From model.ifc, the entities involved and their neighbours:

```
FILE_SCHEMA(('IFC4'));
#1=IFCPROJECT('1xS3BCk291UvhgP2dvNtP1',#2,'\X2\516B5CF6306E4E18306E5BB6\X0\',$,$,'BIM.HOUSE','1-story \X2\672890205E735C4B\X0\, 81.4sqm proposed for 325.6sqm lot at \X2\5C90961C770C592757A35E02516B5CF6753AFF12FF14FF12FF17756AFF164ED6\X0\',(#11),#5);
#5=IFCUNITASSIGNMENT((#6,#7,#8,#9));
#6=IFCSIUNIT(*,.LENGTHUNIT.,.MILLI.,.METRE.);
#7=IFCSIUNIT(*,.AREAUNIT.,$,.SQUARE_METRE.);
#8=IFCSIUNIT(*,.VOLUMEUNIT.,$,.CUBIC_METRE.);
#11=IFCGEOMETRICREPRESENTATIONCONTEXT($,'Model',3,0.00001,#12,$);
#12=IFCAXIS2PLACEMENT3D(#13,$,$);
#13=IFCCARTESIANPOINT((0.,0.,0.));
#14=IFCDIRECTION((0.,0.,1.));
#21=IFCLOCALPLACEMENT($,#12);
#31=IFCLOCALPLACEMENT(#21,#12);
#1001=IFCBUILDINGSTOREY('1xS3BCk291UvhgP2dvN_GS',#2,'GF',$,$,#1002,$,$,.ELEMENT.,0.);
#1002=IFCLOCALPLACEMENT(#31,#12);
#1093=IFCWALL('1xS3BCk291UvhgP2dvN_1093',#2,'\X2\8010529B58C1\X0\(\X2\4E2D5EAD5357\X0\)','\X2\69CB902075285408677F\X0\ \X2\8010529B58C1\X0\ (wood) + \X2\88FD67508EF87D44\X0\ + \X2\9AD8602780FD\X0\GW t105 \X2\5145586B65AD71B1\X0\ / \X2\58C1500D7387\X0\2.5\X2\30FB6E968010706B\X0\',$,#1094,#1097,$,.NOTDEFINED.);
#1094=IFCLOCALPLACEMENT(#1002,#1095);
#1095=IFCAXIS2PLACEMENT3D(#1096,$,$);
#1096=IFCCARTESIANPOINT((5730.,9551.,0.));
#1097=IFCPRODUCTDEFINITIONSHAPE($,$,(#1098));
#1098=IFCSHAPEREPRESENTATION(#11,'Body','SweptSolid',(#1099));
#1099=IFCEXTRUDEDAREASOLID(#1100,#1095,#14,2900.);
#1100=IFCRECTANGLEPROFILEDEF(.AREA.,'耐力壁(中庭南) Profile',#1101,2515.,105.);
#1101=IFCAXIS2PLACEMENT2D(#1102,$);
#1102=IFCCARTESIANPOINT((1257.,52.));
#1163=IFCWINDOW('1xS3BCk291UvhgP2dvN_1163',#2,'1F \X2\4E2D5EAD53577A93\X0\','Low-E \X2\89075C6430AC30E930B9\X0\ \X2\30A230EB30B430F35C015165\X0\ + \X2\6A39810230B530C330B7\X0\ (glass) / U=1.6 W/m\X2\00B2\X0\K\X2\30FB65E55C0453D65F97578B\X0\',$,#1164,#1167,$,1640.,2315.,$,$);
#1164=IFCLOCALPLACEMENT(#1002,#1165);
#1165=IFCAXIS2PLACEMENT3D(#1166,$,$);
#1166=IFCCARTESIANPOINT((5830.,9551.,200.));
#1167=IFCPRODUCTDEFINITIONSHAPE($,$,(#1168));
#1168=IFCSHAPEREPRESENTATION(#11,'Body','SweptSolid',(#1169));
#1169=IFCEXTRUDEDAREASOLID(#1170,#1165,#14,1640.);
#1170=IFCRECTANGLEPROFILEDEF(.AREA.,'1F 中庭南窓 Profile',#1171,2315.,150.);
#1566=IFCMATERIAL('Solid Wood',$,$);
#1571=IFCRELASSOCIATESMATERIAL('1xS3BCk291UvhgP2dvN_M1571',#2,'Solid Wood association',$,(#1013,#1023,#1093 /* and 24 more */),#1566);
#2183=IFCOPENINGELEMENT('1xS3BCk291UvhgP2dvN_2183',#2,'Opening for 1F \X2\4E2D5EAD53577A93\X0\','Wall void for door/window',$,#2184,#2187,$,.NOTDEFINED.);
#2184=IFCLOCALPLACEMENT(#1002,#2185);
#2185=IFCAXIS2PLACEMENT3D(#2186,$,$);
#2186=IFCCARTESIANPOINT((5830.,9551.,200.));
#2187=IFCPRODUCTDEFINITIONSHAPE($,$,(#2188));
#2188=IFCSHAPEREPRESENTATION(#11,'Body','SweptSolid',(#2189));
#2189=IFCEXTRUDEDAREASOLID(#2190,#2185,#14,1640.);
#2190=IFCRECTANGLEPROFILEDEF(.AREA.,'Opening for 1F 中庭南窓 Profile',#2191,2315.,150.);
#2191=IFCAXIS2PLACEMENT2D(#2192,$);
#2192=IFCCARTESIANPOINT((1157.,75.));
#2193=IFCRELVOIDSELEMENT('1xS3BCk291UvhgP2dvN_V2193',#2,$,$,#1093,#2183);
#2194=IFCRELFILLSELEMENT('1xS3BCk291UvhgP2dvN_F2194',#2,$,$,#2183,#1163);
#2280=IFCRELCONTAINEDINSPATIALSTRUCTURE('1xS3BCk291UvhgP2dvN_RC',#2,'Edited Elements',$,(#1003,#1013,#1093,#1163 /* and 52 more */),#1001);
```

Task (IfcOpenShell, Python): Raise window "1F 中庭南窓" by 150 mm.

```python
import numpy as np
import ifcopenshell
import ifcopenshell.api.geometry
import ifcopenshell.util.placement
import ifcopenshell.util.unit

model = ifcopenshell.open("model.ifc")
unit_scale = ifcopenshell.util.unit.calculate_unit_scale(model)

window = model.by_guid("1xS3BCk291UvhgP2dvN_1163")
opening = window.FillsVoids[0].RelatingOpeningElement
dz = 0.15 / unit_scale

shift = np.array([0.0, 0.0, dz])
# The window is not placed relative to its opening, so move both.
for product in (opening, window):
    matrix = ifcopenshell.util.placement.get_local_placement(product.ObjectPlacement)
    matrix[:3, 3] += shift
    ifcopenshell.api.geometry.edit_object_placement(model, product=product, matrix=matrix, is_si=False)

print(f"moved by {dz * unit_scale:+.3f} m")

model.write("model_rev.ifc")
```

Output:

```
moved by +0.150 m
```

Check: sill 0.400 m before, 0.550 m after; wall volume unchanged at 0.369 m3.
